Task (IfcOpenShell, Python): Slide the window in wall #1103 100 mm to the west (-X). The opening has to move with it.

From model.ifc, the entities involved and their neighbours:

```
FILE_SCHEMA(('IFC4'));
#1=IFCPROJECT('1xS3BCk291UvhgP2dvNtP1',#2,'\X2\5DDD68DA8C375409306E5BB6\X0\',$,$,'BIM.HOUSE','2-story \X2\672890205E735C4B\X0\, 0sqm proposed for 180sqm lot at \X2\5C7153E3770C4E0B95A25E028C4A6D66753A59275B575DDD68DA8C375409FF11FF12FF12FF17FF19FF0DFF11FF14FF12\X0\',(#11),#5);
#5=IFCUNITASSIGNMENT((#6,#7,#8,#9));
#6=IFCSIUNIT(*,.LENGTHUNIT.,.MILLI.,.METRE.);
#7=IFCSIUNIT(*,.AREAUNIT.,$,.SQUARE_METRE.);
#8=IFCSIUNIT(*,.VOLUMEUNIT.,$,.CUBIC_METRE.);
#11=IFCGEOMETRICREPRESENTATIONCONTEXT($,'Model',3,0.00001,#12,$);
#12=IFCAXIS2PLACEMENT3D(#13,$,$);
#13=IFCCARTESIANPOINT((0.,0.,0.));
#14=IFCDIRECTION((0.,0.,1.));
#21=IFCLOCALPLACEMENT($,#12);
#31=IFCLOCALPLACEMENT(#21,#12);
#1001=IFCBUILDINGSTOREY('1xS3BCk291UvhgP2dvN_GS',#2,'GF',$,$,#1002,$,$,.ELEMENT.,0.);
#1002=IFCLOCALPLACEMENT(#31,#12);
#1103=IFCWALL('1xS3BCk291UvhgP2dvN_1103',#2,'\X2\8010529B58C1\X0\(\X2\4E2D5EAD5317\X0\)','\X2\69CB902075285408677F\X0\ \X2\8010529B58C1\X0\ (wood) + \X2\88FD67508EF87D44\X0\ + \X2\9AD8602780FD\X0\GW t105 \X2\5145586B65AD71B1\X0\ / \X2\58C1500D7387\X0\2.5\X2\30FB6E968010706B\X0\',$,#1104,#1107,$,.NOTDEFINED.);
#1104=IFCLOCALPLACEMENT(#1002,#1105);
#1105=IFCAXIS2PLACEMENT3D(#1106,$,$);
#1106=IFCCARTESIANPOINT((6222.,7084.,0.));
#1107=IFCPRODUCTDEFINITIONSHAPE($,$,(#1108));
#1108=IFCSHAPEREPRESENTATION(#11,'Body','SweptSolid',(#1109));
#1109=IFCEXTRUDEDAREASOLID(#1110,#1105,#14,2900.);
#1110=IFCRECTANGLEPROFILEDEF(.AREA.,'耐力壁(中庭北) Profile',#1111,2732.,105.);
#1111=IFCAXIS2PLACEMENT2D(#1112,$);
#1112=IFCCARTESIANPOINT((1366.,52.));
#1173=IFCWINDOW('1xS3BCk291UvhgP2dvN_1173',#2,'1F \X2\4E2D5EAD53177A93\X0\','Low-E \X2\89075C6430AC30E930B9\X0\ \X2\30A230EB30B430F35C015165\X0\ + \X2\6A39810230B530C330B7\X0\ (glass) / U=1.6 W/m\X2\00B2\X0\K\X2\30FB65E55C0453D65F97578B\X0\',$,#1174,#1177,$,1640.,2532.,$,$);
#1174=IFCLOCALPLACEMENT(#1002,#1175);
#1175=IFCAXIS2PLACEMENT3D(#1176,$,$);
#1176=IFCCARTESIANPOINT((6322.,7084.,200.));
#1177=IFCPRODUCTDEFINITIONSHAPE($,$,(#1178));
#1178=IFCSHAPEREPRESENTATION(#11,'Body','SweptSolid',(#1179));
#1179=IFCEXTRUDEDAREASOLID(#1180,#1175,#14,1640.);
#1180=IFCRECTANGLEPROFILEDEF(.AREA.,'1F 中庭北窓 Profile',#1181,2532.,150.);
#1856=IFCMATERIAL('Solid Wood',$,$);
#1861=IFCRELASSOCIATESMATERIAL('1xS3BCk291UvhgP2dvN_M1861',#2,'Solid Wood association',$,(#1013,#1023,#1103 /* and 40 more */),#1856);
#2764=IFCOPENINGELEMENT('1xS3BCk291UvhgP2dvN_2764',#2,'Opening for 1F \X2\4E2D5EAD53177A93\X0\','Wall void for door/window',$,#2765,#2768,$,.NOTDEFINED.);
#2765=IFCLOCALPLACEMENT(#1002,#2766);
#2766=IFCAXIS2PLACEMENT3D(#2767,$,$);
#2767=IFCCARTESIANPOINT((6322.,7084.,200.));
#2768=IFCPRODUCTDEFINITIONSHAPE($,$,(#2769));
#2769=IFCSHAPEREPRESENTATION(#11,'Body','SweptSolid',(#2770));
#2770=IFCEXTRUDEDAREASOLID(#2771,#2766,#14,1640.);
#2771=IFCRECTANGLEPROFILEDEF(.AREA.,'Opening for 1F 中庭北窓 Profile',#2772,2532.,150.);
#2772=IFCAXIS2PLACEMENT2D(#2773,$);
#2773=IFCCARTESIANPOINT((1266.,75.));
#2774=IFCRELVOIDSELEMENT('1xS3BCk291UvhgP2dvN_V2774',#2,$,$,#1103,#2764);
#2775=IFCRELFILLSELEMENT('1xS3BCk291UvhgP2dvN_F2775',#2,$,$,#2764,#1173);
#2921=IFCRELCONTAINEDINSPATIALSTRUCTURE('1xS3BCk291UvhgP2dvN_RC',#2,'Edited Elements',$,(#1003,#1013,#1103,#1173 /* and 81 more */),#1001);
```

```python
import ifcopenshell
import ifcopenshell.api.geometry
import ifcopenshell.util.placement
import ifcopenshell.util.unit

model = ifcopenshell.open("model.ifc")
unit_scale = ifcopenshell.util.unit.calculate_unit_scale(model)

window = model.by_guid("1xS3BCk291UvhgP2dvN_1173")
opening = window.FillsVoids[0].RelatingOpeningElement
wall = opening.VoidsElements[0].RelatingBuildingElement

wall_matrix = ifcopenshell.util.placement.get_local_placement(wall.ObjectPlacement)
shift = wall_matrix[:3, 0] * -0.1 / unit_scale
before = ifcopenshell.util.placement.get_local_placement(window.ObjectPlacement)[:3, 3].copy()

# The window is not placed relative to its opening, so move both.
for product in (opening, window):
    matrix = ifcopenshell.util.placement.get_local_placement(product.ObjectPlacement)
    matrix[:3, 3] += shift
    ifcopenshell.api.geometry.edit_object_placement(model, product=product, matrix=matrix, is_si=False)

after = ifcopenshell.util.placement.get_local_placement(window.ObjectPlacement)[:3, 3]
print("window moved by", (after - before).round(3) + 0.0)

model.write("model-out.ifc")
```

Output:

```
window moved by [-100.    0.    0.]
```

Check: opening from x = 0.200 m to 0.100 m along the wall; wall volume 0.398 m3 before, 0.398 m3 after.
